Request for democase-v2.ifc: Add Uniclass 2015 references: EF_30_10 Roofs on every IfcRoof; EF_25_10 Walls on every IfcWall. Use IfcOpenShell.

First a look at what the model holds.

```python
import ifcopenshell

model = ifcopenshell.open("democase-v2.ifc")
print(model.schema)
print("classifications:", [c.Name for c in model.by_type("IfcClassification")])
for ifc_class in ("IfcDoor", "IfcRoof", "IfcStair", "IfcWall", "IfcWindow"):
    print(ifc_class, len(model.by_type(ifc_class)))
```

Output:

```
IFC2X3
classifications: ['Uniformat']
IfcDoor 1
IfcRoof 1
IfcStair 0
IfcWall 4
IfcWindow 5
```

```python
import ifcopenshell
import ifcopenshell.api.classification

model = ifcopenshell.open("democase-v2.ifc")

# IFC2X3 requires Source and Edition and has no link from the project to the system.
system = model.create_entity("IfcClassification", Source="NBS", Edition="2015", Name="Uniclass 2015")

codes = {
    "IfcRoof": ("EF_30_10", "Roofs"),
    "IfcWall": ("EF_25_10", "Walls"),
}
for ifc_class, (code, name) in codes.items():
    products = model.by_type(ifc_class)
    ifcopenshell.api.classification.add_reference(
        model, products=products, classification=system, identification=code, name=name
    )
    print(code, len(products))

model.write("democase-v2_rev.ifc")
```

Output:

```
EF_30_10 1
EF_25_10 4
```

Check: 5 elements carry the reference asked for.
